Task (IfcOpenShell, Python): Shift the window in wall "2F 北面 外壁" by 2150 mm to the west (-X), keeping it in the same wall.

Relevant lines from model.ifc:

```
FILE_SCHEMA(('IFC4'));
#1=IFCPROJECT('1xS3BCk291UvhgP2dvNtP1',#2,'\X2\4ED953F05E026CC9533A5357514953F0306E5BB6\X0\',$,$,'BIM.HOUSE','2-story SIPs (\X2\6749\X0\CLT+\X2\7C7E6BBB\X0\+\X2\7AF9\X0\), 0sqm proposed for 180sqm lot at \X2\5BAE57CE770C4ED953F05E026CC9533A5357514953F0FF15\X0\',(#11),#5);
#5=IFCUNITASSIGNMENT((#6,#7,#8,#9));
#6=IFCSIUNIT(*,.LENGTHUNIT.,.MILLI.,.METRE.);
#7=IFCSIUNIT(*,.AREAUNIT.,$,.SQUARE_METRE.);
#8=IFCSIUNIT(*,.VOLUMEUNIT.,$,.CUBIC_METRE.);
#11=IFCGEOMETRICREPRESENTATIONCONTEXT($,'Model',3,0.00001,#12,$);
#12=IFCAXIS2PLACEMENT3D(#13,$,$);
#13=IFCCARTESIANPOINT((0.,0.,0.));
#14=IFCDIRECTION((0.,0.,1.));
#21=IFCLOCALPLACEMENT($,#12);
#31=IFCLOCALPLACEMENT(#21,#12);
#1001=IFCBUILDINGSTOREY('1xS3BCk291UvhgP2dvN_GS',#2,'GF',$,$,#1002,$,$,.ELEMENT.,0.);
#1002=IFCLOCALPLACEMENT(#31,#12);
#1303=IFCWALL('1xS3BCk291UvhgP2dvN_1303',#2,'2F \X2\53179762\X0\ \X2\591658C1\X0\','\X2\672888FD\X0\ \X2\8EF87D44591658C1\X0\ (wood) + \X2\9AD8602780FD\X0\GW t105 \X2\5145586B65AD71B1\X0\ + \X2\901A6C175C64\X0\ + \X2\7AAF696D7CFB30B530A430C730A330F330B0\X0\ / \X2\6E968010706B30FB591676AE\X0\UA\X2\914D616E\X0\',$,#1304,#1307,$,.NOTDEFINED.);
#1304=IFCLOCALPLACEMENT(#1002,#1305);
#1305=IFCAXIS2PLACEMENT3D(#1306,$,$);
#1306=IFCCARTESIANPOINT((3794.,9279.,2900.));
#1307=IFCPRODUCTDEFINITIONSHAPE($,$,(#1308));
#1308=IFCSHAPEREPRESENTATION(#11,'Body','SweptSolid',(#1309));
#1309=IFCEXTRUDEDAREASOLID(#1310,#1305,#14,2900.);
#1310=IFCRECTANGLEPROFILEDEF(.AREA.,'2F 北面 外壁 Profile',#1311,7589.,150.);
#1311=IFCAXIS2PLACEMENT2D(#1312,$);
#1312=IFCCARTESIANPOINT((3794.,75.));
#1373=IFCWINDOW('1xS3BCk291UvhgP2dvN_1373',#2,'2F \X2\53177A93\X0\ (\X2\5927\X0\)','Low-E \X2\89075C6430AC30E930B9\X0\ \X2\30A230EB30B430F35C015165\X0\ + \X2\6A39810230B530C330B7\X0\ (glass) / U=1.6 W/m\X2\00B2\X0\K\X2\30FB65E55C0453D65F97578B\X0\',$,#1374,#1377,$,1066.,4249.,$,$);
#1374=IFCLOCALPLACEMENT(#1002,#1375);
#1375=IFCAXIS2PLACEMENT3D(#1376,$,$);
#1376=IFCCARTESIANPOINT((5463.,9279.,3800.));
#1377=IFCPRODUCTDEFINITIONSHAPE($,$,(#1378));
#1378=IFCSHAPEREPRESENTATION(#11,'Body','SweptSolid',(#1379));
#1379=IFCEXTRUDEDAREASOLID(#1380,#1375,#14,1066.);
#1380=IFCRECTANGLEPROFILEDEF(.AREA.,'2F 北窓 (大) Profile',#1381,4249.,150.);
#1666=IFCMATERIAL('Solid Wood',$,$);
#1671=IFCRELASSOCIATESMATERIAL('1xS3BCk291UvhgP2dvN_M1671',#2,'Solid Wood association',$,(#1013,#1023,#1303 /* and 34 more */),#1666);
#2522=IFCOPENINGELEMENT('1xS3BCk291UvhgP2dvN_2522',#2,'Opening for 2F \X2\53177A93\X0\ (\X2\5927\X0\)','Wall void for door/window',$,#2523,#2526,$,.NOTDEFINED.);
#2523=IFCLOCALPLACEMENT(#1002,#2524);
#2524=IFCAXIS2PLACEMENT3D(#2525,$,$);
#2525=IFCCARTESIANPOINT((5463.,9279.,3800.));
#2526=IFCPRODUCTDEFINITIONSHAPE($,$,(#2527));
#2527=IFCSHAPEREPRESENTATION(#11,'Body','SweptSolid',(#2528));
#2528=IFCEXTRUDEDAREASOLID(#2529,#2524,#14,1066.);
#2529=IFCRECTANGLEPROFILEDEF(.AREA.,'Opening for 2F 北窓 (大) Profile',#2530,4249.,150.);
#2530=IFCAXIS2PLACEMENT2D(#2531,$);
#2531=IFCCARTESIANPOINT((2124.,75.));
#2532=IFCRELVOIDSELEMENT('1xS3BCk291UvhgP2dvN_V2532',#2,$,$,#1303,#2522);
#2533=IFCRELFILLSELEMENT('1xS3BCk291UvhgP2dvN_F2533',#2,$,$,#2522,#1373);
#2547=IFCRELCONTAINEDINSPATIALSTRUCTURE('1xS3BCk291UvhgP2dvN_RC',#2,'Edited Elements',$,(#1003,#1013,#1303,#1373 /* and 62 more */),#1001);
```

```python
import ifcopenshell
import ifcopenshell.api.geometry
import ifcopenshell.util.placement

model = ifcopenshell.open("model.ifc")

window = model.by_guid("1xS3BCk291UvhgP2dvN_1373")
opening = window.FillsVoids[0].RelatingOpeningElement
wall = opening.VoidsElements[0].RelatingBuildingElement

wall_matrix = ifcopenshell.util.placement.get_local_placement(wall.ObjectPlacement)
shift = wall_matrix[:3, 0] * -2150.0
before = ifcopenshell.util.placement.get_local_placement(window.ObjectPlacement)[:3, 3].copy()

# The window is not placed relative to its opening, so move both.
for product in (opening, window):
    matrix = ifcopenshell.util.placement.get_local_placement(product.ObjectPlacement)
    matrix[:3, 3] += shift
    ifcopenshell.api.geometry.edit_object_placement(model, product=product, matrix=matrix, is_si=False)

after = ifcopenshell.util.placement.get_local_placement(window.ObjectPlacement)[:3, 3]
print("window moved by", (after - before).round(3) + 0.0)

model.write("model-out.ifc")
```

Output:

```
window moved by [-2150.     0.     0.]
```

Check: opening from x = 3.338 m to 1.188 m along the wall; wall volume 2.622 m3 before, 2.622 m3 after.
